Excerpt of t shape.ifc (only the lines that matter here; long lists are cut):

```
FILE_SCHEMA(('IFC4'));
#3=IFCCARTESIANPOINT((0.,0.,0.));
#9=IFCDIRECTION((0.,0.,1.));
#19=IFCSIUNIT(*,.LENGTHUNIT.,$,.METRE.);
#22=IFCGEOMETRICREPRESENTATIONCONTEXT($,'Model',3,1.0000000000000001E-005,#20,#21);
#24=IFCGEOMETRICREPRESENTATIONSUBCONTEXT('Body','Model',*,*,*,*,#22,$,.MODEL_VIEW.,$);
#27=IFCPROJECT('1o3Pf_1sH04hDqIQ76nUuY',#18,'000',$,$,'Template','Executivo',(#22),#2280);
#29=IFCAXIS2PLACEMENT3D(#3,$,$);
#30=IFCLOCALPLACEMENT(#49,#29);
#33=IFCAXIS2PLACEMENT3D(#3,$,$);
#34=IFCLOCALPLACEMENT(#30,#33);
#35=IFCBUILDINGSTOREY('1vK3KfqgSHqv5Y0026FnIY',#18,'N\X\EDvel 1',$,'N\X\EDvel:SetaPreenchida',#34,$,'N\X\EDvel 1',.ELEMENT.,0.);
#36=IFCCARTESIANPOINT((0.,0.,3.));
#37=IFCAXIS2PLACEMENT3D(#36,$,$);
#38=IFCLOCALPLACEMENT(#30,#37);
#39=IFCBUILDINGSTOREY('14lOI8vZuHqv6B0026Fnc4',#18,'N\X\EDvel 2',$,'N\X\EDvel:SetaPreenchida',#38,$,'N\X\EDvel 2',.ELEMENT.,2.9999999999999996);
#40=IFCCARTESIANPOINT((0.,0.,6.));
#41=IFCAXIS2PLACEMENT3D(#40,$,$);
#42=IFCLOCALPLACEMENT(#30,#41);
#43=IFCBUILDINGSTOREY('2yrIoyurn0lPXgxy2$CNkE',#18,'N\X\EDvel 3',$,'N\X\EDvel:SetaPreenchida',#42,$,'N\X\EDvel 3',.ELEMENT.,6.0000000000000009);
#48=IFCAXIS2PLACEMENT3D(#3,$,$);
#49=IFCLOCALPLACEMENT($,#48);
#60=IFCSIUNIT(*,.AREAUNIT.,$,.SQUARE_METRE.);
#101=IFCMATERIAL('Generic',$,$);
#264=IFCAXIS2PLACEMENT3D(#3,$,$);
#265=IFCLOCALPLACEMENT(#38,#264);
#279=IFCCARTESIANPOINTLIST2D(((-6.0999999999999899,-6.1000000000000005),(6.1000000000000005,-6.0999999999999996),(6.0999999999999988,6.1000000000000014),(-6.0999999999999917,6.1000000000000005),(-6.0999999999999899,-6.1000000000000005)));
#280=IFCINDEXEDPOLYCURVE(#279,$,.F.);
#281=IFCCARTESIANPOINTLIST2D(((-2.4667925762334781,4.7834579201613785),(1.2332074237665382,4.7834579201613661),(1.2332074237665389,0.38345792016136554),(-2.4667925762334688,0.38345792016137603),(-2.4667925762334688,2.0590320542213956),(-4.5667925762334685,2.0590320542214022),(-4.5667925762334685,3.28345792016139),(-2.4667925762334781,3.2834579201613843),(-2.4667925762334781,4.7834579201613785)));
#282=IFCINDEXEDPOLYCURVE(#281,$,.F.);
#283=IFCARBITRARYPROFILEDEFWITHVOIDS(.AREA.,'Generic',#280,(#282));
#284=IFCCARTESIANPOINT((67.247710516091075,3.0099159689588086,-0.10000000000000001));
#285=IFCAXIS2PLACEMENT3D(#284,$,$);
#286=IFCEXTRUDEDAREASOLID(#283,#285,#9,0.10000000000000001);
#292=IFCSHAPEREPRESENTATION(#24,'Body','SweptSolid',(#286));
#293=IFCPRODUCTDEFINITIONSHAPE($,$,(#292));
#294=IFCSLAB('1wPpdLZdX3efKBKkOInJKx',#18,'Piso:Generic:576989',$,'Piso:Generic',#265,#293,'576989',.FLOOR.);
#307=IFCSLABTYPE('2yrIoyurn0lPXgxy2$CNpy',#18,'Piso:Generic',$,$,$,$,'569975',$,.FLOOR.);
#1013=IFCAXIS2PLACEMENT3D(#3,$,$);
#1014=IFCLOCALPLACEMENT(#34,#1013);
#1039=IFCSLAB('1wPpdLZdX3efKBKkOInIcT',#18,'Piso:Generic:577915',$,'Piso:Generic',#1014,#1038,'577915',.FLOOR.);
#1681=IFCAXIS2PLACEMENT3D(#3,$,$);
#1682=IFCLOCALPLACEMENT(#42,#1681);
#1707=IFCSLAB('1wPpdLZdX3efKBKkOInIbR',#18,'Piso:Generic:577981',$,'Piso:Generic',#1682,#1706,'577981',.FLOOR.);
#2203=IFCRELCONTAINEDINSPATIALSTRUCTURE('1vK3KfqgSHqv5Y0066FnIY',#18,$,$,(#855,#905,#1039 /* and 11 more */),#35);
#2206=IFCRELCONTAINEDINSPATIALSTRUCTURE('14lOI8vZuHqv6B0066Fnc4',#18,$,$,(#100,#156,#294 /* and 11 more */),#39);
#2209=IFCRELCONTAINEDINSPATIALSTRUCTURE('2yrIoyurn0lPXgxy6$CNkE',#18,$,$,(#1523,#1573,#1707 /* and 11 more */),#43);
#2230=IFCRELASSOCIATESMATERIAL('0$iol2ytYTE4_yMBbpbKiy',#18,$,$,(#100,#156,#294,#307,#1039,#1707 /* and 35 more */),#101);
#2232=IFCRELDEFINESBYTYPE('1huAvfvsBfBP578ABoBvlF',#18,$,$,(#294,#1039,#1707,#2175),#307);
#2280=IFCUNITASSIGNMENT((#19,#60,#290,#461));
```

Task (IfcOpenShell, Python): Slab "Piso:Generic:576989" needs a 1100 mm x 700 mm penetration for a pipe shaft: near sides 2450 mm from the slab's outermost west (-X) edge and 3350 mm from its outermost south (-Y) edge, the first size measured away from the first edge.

```python
import numpy as np
import ifcopenshell
import ifcopenshell.api.feature
import ifcopenshell.api.geometry
import ifcopenshell.api.root
import ifcopenshell.geom
import ifcopenshell.util.placement
import ifcopenshell.util.representation
import ifcopenshell.util.shape
import ifcopenshell.util.unit

model = ifcopenshell.open("t shape.ifc")
unit_scale = ifcopenshell.util.unit.calculate_unit_scale(model)
settings = ifcopenshell.geom.settings()


def volume(element):
    """Net volume in cubic metres, openings subtracted."""
    shape = ifcopenshell.geom.create_shape(settings, element)
    return ifcopenshell.util.shape.get_volume(shape.geometry)


slab = model.by_guid("1wPpdLZdX3efKBKkOInJKx")
before = volume(slab)

# Extent in the slab's own axes, in metres. The edges named are its -X and -Y sides.
slab_shape = ifcopenshell.geom.create_shape(settings, slab)
vertices = ifcopenshell.util.shape.get_vertices(slab_shape.geometry)
x_min, y_min, bottom = vertices.min(axis=0)
top = vertices[:, 2].max()

opening = ifcopenshell.api.root.create_entity(model, ifc_class="IfcOpeningElement", name="Pipe shaft opening", predefined_type="OPENING")
context = ifcopenshell.util.representation.get_context(model, "Model", "Body", "MODEL_VIEW")
width, depth = 1.1, 0.7
outline = [(0.0, 0.0), (width, 0.0), (width, depth), (0.0, depth), (0.0, 0.0)]
# Overshoot both faces by 50 mm so the cut is clean.
shape = ifcopenshell.api.geometry.add_slab_representation(
    model, context=context, depth=top - bottom + 0.1, polyline=outline
)
ifcopenshell.api.geometry.assign_representation(model, product=opening, representation=shape)

matrix = ifcopenshell.util.placement.get_local_placement(slab.ObjectPlacement)
matrix[:, 3] = matrix @ np.append(np.array([x_min + 2.45, y_min + 3.35, bottom - 0.05]) / unit_scale, 1.0)
ifcopenshell.api.geometry.edit_object_placement(model, product=opening, matrix=matrix, is_si=False)
ifcopenshell.api.feature.add_feature(model, feature=opening, element=slab)

after = volume(slab)

print(f"slab volume {before:.3f} -> {after:.3f} m3")

model.write("t shape_v2.ifc")
```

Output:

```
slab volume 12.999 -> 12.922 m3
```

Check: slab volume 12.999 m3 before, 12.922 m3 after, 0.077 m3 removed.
